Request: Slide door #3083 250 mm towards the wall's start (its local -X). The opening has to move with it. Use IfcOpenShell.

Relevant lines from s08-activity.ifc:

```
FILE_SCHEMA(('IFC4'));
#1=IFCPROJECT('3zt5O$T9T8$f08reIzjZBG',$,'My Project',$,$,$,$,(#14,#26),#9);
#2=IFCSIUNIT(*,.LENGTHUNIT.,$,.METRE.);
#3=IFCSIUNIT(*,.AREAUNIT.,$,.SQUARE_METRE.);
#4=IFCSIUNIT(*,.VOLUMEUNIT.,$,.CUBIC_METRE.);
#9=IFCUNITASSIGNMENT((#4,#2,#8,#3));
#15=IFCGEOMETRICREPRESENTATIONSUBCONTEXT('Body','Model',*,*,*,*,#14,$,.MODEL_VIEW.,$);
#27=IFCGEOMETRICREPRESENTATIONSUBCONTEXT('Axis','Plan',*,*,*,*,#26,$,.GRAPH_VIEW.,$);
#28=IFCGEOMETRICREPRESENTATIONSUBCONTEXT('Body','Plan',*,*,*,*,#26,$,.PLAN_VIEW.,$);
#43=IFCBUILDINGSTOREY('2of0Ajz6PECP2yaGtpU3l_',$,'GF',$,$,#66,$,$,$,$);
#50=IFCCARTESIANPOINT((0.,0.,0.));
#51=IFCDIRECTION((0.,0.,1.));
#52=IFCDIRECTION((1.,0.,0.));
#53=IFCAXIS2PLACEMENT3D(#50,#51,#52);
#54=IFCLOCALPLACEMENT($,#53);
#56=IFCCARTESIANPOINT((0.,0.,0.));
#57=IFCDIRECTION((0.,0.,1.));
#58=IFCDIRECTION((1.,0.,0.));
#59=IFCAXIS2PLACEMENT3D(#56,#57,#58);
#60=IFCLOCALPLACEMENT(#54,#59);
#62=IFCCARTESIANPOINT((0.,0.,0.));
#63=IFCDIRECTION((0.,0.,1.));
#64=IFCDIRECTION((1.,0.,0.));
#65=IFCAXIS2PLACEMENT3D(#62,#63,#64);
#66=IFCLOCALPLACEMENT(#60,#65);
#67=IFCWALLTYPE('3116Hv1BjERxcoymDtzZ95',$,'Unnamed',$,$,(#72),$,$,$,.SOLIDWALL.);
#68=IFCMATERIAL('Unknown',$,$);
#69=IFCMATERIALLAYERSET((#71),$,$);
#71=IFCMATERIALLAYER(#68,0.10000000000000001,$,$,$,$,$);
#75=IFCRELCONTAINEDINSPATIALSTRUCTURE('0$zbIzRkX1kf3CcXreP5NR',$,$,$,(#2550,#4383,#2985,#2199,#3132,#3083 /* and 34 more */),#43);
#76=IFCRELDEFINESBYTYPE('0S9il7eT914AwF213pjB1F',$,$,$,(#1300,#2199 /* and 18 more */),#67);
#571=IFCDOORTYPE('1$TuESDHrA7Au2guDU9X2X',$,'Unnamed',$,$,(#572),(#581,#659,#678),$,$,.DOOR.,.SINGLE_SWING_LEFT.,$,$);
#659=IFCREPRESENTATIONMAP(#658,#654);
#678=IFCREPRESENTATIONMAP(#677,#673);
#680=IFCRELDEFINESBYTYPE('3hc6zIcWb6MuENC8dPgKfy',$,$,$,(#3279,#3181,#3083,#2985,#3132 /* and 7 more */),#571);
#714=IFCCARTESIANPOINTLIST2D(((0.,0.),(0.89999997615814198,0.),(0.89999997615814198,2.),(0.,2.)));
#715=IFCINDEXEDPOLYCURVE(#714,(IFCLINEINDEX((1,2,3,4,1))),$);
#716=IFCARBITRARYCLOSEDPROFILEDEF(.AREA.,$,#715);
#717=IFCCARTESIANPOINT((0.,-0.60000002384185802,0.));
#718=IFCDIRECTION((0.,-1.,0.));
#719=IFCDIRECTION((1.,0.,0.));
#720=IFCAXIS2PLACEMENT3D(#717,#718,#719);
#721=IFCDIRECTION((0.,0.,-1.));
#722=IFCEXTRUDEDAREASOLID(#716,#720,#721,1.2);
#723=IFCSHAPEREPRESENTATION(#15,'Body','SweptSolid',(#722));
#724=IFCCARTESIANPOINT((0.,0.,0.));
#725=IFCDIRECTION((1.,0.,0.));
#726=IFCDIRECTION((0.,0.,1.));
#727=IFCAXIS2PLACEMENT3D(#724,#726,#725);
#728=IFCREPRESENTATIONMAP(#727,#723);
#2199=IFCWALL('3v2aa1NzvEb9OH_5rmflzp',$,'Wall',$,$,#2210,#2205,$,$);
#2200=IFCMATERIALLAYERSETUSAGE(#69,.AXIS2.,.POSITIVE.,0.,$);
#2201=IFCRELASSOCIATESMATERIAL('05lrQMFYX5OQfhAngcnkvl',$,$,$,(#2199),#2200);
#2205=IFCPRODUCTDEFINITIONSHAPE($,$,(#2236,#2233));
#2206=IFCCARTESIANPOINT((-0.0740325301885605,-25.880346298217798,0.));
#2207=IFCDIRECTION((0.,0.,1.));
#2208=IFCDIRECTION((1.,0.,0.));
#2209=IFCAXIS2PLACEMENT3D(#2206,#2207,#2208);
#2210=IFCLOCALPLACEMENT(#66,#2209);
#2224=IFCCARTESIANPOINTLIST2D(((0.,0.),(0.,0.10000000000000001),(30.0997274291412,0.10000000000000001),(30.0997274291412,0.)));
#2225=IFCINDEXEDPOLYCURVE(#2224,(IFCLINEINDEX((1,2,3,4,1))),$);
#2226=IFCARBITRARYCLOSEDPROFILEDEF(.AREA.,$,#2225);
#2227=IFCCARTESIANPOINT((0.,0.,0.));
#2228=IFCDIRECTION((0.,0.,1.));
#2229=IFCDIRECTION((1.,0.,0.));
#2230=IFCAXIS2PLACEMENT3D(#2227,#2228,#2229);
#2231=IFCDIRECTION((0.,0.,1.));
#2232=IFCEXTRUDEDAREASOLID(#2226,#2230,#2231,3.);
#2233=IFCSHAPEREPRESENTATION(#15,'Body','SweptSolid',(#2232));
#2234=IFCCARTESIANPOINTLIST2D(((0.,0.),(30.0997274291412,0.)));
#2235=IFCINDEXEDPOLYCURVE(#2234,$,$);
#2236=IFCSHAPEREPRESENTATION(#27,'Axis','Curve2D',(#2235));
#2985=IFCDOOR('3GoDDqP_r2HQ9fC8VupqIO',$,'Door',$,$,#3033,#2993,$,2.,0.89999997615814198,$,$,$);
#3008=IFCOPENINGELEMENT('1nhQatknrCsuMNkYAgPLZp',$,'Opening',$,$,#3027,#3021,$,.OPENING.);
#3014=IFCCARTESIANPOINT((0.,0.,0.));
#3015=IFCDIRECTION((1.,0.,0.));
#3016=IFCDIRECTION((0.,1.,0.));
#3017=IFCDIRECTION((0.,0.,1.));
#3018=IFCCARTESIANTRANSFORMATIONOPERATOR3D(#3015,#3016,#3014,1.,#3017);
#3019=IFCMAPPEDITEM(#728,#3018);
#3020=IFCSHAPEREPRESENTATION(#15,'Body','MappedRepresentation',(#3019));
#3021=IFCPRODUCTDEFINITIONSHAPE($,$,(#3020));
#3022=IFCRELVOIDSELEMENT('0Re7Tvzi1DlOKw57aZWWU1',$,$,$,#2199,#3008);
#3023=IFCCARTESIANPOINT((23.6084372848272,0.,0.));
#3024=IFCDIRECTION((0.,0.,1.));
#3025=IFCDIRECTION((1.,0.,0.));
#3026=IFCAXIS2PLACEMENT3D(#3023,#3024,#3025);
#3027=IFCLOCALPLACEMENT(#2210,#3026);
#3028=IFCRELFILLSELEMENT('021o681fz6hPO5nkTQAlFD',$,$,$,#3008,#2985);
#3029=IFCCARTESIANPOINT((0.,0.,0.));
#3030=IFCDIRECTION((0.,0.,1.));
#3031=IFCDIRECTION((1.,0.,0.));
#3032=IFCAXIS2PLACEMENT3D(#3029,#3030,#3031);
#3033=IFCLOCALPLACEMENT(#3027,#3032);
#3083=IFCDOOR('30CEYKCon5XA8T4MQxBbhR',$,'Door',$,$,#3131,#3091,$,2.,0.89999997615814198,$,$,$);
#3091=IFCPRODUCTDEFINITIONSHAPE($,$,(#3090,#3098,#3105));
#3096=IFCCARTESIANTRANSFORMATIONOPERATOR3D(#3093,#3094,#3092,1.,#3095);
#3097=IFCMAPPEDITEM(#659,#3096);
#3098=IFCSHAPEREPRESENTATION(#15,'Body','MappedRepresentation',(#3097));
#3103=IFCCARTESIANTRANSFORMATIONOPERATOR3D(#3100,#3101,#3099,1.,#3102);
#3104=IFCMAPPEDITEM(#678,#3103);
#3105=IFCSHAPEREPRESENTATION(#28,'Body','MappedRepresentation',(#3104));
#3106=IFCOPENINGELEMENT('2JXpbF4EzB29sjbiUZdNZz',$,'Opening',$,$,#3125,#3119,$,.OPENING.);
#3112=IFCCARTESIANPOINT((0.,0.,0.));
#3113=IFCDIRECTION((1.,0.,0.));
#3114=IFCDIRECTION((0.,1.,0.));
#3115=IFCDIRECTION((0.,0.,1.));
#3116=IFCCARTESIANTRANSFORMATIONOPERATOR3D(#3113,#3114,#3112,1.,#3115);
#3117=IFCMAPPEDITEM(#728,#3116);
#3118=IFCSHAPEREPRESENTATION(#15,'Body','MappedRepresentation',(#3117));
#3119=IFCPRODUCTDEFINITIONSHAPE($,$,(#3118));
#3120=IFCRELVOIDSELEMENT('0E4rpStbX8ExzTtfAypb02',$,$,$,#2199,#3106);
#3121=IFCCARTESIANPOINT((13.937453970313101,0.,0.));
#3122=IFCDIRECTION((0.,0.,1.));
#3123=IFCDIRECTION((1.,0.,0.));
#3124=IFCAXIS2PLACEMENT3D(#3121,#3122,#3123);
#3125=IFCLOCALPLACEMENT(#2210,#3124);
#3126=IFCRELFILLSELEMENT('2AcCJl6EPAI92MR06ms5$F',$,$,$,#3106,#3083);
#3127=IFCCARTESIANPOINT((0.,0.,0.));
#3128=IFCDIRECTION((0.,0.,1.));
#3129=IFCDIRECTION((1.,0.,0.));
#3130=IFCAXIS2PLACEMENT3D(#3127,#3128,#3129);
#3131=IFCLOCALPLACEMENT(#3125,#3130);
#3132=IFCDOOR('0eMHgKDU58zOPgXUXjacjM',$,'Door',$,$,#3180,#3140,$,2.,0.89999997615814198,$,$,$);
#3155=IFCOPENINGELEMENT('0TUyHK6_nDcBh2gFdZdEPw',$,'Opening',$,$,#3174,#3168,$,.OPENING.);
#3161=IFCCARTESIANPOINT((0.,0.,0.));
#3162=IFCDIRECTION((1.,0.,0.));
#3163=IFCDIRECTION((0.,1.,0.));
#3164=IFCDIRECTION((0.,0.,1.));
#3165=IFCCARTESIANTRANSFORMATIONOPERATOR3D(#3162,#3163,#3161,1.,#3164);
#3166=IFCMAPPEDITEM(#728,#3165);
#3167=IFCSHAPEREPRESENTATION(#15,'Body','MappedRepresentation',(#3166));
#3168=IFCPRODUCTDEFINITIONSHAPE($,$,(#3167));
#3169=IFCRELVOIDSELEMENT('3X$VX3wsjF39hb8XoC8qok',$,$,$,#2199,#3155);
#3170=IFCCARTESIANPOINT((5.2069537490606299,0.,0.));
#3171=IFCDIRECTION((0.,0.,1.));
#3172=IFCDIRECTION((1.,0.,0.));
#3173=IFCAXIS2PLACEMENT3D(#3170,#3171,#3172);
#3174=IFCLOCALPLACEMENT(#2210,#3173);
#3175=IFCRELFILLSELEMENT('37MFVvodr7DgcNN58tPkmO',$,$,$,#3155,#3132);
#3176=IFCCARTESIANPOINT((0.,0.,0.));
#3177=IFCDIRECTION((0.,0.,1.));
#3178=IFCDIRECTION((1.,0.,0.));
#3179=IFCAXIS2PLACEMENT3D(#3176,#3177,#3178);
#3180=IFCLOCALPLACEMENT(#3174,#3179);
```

```python
import ifcopenshell
import ifcopenshell.api.geometry
import ifcopenshell.util.placement
import ifcopenshell.util.unit

model = ifcopenshell.open("s08-activity.ifc")
unit_scale = ifcopenshell.util.unit.calculate_unit_scale(model)

door = model.by_guid("30CEYKCon5XA8T4MQxBbhR")
opening = door.FillsVoids[0].RelatingOpeningElement
wall = opening.VoidsElements[0].RelatingBuildingElement

wall_matrix = ifcopenshell.util.placement.get_local_placement(wall.ObjectPlacement)
shift = wall_matrix[:3, 0] * -0.25 / unit_scale
before = ifcopenshell.util.placement.get_local_placement(door.ObjectPlacement)[:3, 3].copy()

# The door is placed relative to its opening, so it follows when the opening moves.
matrix = ifcopenshell.util.placement.get_local_placement(opening.ObjectPlacement)
matrix[:3, 3] += shift
ifcopenshell.api.geometry.edit_object_placement(
    model, product=opening, matrix=matrix, is_si=False, should_transform_children=True
)

after = ifcopenshell.util.placement.get_local_placement(door.ObjectPlacement)[:3, 3]
print("door moved by", (after - before).round(3) + 0.0)

model.write("s08-activity_rev.ifc")
```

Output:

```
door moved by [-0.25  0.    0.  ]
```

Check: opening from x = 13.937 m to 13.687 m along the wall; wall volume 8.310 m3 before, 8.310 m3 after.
